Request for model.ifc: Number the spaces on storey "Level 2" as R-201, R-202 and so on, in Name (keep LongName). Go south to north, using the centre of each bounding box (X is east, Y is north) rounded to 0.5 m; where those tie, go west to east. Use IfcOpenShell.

First a look at what the model holds.

```python
import ifcopenshell
import ifcopenshell.util.element
import ifcopenshell.util.placement

model = ifcopenshell.open("model.ifc")
print(model.schema)
storey = next(s for s in model.by_type("IfcBuildingStorey") if s.Name == "Level 2")
spaces = [e for e in ifcopenshell.util.element.get_decomposition(storey) if e.is_a("IfcSpace")]
for e in sorted(spaces, key=lambda e: e.id()):
    origin = ifcopenshell.util.placement.get_local_placement(e.ObjectPlacement)[:3, 3]
    print(e.id(), e.Name, e.LongName, origin.round(2) + 0.0, sep=" | ")
```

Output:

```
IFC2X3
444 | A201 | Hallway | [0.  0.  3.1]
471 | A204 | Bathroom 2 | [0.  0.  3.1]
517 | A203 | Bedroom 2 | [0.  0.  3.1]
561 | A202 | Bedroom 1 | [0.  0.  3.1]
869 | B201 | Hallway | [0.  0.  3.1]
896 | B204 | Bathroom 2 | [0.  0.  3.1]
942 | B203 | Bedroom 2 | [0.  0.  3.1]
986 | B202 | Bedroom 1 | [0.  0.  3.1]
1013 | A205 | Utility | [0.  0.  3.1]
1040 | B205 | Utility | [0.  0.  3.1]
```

```python
import ifcopenshell
import ifcopenshell.geom
import ifcopenshell.util.element
import ifcopenshell.util.shape

model = ifcopenshell.open("model.ifc")
settings = ifcopenshell.geom.settings()
settings.set("use-world-coords", True)


def centre(element):
    shape = ifcopenshell.geom.create_shape(settings, element)
    return ifcopenshell.util.shape.get_bbox_centroid(shape.geometry)


storey = next(s for s in model.by_type("IfcBuildingStorey") if s.Name == "Level 2")
spaces = [e for e in ifcopenshell.util.element.get_decomposition(storey) if e.is_a("IfcSpace")]

# Insertion points can sit at a corner or the storey origin, so sort by the geometry (in metres).
centres = {e: centre(e) for e in spaces}
spaces.sort(key=lambda e: (round(centres[e][1] / 0.5), centres[e][0]))

for i, e in enumerate(spaces, start=1):
    number = f"R-2{i:02d}"
    e.Name = number
    print(e.id(), number)

model.write("model_v2.ifc")
```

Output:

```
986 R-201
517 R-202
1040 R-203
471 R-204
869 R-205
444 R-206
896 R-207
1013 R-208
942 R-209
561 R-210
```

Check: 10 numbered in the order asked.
